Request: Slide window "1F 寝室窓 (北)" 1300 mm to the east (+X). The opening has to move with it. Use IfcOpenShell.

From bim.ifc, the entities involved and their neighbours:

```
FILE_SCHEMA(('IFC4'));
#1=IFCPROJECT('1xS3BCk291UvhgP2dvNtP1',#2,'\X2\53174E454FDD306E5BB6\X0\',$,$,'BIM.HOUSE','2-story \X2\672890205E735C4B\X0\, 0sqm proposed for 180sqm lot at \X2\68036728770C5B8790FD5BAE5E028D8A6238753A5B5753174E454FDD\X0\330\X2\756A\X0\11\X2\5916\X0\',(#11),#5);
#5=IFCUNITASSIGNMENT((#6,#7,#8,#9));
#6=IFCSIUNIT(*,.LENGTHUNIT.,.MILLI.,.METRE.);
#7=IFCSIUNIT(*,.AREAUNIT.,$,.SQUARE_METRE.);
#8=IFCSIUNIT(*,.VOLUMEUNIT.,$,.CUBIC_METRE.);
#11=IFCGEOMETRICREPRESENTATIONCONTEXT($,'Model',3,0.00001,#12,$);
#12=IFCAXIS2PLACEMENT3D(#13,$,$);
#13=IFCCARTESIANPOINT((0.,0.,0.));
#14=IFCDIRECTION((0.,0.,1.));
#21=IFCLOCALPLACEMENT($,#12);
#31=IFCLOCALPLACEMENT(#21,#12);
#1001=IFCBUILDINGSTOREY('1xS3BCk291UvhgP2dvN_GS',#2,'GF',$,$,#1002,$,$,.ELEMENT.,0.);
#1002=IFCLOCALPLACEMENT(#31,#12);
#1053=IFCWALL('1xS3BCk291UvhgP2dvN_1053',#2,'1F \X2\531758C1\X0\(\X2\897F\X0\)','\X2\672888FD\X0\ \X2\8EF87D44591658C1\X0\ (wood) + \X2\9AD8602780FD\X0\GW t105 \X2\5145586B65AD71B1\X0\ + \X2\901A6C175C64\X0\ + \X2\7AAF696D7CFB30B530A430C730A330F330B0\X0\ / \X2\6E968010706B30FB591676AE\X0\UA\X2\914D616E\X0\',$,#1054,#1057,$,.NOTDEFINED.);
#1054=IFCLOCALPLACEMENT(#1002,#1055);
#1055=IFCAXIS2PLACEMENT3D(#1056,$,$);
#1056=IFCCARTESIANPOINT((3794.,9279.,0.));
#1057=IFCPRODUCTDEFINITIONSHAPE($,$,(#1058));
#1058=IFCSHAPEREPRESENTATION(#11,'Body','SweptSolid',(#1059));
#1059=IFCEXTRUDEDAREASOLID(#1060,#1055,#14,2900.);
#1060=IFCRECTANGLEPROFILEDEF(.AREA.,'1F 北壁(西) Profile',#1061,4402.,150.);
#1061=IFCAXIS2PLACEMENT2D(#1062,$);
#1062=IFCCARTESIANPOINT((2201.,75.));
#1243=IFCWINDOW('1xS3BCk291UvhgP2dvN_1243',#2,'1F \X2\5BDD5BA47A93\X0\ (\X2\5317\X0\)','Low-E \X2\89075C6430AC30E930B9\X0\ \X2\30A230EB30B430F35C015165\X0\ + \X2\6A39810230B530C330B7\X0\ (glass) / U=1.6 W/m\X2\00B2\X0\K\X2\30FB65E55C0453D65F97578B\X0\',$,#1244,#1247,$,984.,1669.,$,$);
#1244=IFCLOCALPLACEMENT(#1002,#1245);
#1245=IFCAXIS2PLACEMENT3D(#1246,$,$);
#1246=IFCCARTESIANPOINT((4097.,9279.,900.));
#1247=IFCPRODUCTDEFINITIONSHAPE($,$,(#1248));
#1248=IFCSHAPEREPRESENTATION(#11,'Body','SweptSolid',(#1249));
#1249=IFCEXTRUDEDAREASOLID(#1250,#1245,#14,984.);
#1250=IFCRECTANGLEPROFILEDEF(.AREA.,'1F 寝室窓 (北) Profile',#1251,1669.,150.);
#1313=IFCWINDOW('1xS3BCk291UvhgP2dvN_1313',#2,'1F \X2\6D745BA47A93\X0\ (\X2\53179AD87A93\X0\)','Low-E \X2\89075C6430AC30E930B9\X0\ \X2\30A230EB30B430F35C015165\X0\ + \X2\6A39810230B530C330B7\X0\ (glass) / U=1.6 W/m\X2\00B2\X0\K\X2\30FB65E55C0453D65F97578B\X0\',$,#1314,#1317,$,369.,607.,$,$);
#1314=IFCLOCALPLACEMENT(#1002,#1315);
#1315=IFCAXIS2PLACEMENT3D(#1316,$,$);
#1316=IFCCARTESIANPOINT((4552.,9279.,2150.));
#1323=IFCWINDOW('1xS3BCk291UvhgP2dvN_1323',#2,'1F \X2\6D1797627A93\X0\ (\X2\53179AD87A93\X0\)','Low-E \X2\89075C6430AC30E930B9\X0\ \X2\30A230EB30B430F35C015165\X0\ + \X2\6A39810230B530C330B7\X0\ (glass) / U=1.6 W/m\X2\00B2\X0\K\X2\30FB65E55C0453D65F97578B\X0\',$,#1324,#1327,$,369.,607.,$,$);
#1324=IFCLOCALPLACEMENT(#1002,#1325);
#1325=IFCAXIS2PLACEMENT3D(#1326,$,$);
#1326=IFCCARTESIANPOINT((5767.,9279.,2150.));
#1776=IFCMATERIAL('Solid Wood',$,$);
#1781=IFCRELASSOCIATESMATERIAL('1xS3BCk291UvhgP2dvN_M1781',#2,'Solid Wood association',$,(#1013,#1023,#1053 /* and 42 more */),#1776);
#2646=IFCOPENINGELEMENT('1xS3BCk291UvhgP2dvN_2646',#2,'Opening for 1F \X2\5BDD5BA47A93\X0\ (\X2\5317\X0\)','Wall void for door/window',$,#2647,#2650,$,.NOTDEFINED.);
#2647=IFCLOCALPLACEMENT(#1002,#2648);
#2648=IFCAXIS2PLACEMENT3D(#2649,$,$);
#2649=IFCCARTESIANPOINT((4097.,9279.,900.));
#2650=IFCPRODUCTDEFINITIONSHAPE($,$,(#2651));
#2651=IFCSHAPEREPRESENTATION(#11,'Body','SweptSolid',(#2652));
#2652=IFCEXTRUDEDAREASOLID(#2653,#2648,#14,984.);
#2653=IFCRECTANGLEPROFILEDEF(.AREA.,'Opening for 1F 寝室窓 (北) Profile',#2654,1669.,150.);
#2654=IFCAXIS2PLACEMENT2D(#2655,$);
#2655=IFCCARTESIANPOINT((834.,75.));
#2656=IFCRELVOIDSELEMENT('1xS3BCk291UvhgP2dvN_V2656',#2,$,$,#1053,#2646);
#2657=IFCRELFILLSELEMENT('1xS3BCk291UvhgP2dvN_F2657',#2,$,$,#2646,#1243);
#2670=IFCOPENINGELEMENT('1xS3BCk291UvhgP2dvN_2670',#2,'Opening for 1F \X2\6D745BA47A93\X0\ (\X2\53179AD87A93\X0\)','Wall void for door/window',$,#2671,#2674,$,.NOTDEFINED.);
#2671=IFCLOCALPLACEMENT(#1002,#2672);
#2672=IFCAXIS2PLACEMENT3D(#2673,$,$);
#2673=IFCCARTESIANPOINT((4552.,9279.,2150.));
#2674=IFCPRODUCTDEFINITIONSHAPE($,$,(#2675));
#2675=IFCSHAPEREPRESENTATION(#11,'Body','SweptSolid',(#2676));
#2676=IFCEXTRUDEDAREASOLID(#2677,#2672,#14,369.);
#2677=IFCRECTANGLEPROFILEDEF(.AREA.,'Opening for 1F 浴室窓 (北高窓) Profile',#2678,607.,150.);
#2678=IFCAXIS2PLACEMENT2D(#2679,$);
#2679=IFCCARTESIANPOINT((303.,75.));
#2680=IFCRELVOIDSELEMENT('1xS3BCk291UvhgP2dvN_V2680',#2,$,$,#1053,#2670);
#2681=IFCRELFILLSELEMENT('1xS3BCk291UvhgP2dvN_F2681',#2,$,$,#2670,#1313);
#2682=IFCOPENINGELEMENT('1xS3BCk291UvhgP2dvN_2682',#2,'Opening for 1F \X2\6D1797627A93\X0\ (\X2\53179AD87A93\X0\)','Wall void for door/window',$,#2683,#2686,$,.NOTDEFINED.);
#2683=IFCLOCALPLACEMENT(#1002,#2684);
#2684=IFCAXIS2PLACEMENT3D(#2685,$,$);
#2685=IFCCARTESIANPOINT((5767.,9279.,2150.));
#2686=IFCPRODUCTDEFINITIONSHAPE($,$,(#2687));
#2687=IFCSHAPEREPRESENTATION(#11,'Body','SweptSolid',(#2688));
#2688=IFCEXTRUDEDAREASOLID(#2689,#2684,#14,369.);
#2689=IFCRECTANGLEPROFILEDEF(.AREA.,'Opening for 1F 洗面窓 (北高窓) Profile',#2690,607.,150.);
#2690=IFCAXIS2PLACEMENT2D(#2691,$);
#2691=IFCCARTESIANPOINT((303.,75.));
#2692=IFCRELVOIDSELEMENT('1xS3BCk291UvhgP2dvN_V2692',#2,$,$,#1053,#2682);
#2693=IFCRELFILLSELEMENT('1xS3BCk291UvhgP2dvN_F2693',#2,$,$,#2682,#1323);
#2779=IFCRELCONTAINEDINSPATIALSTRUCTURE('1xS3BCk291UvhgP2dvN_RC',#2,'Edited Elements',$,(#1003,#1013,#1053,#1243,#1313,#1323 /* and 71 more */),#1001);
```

```python
import ifcopenshell
import ifcopenshell.api.geometry
import ifcopenshell.util.placement
import ifcopenshell.util.unit

model = ifcopenshell.open("bim.ifc")
unit_scale = ifcopenshell.util.unit.calculate_unit_scale(model)

window = model.by_guid("1xS3BCk291UvhgP2dvN_1243")
opening = window.FillsVoids[0].RelatingOpeningElement
wall = opening.VoidsElements[0].RelatingBuildingElement

wall_matrix = ifcopenshell.util.placement.get_local_placement(wall.ObjectPlacement)
shift = wall_matrix[:3, 0] * 1.3 / unit_scale
before = ifcopenshell.util.placement.get_local_placement(window.ObjectPlacement)[:3, 3].copy()

# The window is not placed relative to its opening, so move both.
for product in (opening, window):
    matrix = ifcopenshell.util.placement.get_local_placement(product.ObjectPlacement)
    matrix[:3, 3] += shift
    ifcopenshell.api.geometry.edit_object_placement(model, product=product, matrix=matrix, is_si=False)

after = ifcopenshell.util.placement.get_local_placement(window.ObjectPlacement)[:3, 3]
print("window moved by", (after - before).round(3) + 0.0)

model.write("bim_v2.ifc")
```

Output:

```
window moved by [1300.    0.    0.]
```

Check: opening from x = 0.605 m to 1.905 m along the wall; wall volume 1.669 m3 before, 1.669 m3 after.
